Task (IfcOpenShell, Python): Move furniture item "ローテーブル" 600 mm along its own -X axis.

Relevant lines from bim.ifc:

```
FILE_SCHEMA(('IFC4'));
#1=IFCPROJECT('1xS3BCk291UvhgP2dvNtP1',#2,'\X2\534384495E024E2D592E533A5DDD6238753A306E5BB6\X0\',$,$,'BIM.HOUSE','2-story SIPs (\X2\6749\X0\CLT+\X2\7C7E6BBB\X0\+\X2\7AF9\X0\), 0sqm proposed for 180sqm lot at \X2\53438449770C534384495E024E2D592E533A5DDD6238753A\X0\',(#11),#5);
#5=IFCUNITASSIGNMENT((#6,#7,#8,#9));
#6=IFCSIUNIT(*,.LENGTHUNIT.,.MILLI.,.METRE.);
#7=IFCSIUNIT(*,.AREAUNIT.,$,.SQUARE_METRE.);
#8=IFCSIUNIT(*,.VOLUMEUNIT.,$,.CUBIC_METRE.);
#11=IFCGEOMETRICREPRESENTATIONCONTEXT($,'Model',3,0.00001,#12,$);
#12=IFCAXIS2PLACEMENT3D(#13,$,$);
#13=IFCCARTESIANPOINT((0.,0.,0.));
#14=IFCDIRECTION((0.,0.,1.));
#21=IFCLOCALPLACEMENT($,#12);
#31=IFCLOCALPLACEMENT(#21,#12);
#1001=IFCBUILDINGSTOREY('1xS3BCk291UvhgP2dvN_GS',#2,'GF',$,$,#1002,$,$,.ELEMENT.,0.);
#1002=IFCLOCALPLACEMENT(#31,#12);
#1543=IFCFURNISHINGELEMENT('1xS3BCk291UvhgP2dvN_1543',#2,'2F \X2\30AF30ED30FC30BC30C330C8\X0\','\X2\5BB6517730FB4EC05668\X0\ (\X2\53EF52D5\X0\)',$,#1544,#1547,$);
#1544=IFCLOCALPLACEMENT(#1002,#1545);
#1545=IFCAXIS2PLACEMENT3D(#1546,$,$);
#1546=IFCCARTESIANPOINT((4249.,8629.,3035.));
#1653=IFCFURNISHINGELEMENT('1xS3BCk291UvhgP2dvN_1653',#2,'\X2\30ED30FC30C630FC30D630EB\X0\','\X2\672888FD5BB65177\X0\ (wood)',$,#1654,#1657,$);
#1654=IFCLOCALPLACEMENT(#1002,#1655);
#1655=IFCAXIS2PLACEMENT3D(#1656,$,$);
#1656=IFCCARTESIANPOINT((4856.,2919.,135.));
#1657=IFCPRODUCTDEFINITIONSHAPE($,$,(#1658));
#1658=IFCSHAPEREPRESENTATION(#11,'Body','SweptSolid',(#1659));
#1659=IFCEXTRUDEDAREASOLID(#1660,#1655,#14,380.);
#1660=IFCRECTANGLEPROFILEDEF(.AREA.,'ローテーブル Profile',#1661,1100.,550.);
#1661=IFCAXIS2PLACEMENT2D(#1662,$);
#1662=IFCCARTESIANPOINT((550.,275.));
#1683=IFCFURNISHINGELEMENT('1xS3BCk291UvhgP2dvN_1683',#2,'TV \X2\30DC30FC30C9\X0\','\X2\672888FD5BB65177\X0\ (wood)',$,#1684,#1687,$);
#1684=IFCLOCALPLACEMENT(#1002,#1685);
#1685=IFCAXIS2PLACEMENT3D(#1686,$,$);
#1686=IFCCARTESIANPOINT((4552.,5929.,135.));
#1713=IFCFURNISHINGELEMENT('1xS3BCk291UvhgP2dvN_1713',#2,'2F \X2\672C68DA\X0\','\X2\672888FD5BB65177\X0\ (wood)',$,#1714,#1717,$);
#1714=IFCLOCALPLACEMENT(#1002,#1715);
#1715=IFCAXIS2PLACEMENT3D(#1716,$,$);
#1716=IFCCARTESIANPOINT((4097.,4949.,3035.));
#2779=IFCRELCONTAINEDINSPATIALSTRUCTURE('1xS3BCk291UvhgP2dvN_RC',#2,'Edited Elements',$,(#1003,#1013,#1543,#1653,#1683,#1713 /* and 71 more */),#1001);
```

```python
import ifcopenshell
import ifcopenshell.api.geometry
import ifcopenshell.util.placement
import ifcopenshell.util.unit

model = ifcopenshell.open("bim.ifc")
unit_scale = ifcopenshell.util.unit.calculate_unit_scale(model)

item = model.by_id(1653)
matrix = ifcopenshell.util.placement.get_local_placement(item.ObjectPlacement)
matrix[:3, 3] -= matrix[:3, 0] * 0.6 / unit_scale
ifcopenshell.api.geometry.edit_object_placement(model, product=item, matrix=matrix, is_si=False)

print(ifcopenshell.util.placement.get_local_placement(item.ObjectPlacement).round(3) + 0.0)

model.write("bim_v2.ifc")
```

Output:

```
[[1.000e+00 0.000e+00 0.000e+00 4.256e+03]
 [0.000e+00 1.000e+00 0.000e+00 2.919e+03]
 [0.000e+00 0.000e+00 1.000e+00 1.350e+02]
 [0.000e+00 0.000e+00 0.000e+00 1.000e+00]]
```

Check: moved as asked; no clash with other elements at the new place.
